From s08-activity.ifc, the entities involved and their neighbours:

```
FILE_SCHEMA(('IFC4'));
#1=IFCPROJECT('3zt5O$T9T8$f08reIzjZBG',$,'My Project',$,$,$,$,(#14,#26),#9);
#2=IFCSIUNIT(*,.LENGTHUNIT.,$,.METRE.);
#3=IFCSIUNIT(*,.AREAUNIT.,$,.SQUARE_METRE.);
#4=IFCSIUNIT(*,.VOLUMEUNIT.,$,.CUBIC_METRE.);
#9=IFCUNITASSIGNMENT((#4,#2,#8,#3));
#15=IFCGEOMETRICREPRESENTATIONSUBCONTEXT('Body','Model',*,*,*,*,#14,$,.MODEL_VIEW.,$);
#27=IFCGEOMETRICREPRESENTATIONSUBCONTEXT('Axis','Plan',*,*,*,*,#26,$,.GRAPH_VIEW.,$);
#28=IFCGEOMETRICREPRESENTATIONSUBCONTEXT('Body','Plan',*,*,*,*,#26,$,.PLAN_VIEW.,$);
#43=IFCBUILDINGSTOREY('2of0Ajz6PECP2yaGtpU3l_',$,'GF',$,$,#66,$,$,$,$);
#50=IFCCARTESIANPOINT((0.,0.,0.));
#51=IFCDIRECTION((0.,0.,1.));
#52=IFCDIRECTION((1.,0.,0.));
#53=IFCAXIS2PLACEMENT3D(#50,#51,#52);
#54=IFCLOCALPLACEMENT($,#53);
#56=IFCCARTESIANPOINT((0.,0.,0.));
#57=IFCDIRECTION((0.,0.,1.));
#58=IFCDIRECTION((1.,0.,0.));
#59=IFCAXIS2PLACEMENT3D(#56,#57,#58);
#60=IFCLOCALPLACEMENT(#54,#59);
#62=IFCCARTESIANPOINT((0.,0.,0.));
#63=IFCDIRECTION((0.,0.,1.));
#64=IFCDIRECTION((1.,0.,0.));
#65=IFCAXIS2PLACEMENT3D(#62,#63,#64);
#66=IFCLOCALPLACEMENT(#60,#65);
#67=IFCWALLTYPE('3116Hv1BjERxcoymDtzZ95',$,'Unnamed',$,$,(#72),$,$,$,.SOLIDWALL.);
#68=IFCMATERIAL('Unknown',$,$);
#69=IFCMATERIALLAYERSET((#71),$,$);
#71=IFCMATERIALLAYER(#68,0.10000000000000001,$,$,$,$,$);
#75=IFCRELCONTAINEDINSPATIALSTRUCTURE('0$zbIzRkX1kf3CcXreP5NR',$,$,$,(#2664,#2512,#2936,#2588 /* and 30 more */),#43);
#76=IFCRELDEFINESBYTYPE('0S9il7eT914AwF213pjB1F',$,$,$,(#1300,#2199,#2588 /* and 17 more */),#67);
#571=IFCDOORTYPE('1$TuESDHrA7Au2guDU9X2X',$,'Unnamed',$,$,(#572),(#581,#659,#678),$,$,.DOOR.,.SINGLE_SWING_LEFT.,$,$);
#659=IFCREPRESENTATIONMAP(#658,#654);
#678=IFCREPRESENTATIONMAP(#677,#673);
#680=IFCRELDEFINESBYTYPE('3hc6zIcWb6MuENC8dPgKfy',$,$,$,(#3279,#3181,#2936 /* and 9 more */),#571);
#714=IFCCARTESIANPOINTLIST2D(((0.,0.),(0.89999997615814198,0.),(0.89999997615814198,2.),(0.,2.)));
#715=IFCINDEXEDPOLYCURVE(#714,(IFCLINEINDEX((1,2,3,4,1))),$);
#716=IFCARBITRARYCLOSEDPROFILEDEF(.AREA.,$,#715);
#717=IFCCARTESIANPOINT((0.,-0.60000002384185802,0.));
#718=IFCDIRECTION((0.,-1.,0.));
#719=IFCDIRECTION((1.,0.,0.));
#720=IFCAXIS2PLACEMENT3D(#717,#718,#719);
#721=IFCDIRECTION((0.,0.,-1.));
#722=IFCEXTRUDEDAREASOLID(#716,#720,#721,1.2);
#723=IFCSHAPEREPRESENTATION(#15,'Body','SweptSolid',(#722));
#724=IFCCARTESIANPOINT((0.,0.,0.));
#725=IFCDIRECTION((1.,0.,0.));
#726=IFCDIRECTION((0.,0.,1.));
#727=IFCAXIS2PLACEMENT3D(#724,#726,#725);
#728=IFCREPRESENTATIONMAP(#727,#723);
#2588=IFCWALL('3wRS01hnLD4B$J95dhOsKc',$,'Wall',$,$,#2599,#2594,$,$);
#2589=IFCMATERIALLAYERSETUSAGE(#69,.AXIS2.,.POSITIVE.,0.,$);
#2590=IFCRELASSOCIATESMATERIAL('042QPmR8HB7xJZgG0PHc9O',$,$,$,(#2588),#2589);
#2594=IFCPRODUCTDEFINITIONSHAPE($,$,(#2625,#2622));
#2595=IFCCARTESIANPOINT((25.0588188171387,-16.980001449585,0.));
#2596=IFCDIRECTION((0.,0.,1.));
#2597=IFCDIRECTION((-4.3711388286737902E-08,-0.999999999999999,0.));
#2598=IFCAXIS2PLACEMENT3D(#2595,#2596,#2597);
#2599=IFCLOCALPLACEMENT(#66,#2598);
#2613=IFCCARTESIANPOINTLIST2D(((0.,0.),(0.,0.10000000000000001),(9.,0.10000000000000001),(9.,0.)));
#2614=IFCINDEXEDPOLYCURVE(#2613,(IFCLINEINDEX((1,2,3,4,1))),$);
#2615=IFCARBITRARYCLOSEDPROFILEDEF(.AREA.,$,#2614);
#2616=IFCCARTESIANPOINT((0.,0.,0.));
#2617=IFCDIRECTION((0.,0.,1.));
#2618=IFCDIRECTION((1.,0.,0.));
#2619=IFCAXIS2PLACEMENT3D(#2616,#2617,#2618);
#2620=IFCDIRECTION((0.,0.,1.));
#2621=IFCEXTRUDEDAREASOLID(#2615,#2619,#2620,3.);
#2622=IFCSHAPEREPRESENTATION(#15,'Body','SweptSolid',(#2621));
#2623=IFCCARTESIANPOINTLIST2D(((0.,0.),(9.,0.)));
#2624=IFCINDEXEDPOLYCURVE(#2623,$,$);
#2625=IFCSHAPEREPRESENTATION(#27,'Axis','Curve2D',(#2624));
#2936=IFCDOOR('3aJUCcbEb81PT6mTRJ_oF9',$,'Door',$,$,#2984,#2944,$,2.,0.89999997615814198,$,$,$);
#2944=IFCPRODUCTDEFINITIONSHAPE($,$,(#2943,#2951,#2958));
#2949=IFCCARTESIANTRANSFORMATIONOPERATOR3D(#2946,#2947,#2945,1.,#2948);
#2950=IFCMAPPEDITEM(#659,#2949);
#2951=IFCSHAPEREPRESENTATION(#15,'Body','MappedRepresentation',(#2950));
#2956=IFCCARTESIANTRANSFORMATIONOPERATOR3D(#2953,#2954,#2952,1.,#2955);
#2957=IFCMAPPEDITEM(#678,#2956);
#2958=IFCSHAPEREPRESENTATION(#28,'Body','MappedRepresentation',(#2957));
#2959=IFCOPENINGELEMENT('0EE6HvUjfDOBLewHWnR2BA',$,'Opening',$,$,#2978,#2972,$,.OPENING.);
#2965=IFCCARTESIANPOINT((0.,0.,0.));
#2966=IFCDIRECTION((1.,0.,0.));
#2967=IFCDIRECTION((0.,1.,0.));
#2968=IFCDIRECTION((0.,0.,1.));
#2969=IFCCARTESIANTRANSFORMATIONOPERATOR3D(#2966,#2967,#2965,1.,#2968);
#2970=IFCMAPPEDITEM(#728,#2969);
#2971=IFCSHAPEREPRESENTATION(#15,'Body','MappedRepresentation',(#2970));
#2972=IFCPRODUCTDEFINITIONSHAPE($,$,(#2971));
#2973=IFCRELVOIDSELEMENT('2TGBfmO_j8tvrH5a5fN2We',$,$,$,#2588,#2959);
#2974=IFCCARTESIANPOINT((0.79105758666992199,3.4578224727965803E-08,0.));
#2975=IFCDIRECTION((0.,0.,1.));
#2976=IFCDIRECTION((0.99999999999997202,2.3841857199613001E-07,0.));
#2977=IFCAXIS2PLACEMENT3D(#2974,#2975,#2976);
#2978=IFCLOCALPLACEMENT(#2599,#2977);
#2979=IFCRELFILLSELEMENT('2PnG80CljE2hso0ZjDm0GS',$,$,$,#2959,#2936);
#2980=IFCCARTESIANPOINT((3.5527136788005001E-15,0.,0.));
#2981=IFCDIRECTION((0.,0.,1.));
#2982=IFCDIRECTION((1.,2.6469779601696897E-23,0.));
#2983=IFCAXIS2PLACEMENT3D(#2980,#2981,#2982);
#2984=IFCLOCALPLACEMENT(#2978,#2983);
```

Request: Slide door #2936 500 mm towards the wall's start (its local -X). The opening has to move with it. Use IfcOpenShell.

```python
import ifcopenshell
import ifcopenshell.api.geometry
import ifcopenshell.util.placement
import ifcopenshell.util.unit

model = ifcopenshell.open("s08-activity.ifc")
unit_scale = ifcopenshell.util.unit.calculate_unit_scale(model)

door = model.by_guid("3aJUCcbEb81PT6mTRJ_oF9")
opening = door.FillsVoids[0].RelatingOpeningElement
wall = opening.VoidsElements[0].RelatingBuildingElement

wall_matrix = ifcopenshell.util.placement.get_local_placement(wall.ObjectPlacement)
shift = wall_matrix[:3, 0] * -0.5 / unit_scale
before = ifcopenshell.util.placement.get_local_placement(door.ObjectPlacement)[:3, 3].copy()

# The door is placed relative to its opening, so it follows when the opening moves.
matrix = ifcopenshell.util.placement.get_local_placement(opening.ObjectPlacement)
matrix[:3, 3] += shift
ifcopenshell.api.geometry.edit_object_placement(
    model, product=opening, matrix=matrix, is_si=False, should_transform_children=True
)

after = ifcopenshell.util.placement.get_local_placement(door.ObjectPlacement)[:3, 3]
print("door moved by", (after - before).round(3) + 0.0)

model.write("s08-activity_v2.ifc")
```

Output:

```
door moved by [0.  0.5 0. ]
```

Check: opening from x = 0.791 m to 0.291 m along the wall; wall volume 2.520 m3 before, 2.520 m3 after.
